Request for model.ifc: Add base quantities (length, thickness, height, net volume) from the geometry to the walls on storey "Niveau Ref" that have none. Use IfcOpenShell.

First a look at what the model holds.

```python
import ifcopenshell
import ifcopenshell.util.element
import ifcopenshell.util.unit

model = ifcopenshell.open("model.ifc")
print(model.schema)
for unit_type in ("LENGTHUNIT", "AREAUNIT", "VOLUMEUNIT"):
    print(unit_type, ifcopenshell.util.unit.calculate_unit_scale(model, unit_type))
storey = next(s for s in model.by_type("IfcBuildingStorey") if s.Name == "Niveau Ref")
walls = [e for e in ifcopenshell.util.element.get_decomposition(storey) if e.is_a("IfcWall")]
for e in sorted(walls, key=lambda e: e.id()):
    print(e.id(), e.is_a(), e.Name, list(ifcopenshell.util.element.get_psets(e, qtos_only=True)), sep=" | ")
```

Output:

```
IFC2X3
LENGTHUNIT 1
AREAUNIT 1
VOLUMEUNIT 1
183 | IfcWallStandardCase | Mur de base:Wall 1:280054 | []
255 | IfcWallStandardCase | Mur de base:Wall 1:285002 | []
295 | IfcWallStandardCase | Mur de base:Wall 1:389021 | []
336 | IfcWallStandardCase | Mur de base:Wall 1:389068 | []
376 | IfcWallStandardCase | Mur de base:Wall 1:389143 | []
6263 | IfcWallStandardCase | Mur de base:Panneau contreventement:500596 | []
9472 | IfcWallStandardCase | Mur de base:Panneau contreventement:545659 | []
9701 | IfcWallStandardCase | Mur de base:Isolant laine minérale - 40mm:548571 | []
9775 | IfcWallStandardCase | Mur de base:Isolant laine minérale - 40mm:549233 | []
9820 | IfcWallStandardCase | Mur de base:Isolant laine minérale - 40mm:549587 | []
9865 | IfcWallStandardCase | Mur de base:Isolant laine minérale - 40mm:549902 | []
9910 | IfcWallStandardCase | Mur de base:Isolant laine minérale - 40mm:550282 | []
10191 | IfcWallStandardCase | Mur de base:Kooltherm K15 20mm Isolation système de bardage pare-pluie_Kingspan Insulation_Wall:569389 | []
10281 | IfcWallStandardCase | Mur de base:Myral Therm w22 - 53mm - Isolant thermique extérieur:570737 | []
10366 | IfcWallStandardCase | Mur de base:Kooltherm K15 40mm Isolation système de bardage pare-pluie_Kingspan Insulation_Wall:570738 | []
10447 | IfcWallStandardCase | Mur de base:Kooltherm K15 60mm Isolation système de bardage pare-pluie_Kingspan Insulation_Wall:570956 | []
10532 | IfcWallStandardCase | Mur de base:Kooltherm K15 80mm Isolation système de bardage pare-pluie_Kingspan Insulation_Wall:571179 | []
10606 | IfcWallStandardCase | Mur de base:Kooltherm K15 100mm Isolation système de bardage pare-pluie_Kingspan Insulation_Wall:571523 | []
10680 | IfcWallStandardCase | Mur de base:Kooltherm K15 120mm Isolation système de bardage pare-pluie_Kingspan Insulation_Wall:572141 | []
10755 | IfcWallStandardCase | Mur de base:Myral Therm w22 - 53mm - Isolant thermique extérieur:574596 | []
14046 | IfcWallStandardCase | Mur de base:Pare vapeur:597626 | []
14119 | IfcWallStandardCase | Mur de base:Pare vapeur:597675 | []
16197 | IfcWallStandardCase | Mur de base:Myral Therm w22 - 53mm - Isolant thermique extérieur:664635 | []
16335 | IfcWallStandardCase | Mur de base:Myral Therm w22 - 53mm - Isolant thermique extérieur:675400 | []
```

```python
import ifcopenshell
import ifcopenshell.api.pset
import ifcopenshell.geom
import ifcopenshell.util.element
import ifcopenshell.util.shape
import ifcopenshell.util.unit

model = ifcopenshell.open("model.ifc")
unit_scale = ifcopenshell.util.unit.calculate_unit_scale(model)
volume_scale = ifcopenshell.util.unit.calculate_unit_scale(model, "VOLUMEUNIT")
settings = ifcopenshell.geom.settings()

storey = next(s for s in model.by_type("IfcBuildingStorey") if s.Name == "Niveau Ref")
walls = [e for e in ifcopenshell.util.element.get_decomposition(storey) if e.is_a("IfcWall")]

for e in sorted(walls, key=lambda e: e.id()):
    if ifcopenshell.util.element.get_psets(e, qtos_only=True, should_inherit=False):
        continue
    # Geometry comes back in metres, in the element's own axes.
    shape = ifcopenshell.geom.create_shape(settings, e)
    values = {
        "Length": ifcopenshell.util.shape.get_x(shape.geometry) / unit_scale,
        "Width": ifcopenshell.util.shape.get_y(shape.geometry) / unit_scale,
        "Height": ifcopenshell.util.shape.get_z(shape.geometry) / unit_scale,
        "NetVolume": ifcopenshell.util.shape.get_volume(shape.geometry) / volume_scale,
    }
    qto = ifcopenshell.api.pset.add_qto(model, product=e, name="BaseQuantities")
    ifcopenshell.api.pset.edit_qto(model, qto=qto, properties=values)
    print(e.id(), {k: round(v, 3) for k, v in values.items()})

model.write("model-out.ifc")
```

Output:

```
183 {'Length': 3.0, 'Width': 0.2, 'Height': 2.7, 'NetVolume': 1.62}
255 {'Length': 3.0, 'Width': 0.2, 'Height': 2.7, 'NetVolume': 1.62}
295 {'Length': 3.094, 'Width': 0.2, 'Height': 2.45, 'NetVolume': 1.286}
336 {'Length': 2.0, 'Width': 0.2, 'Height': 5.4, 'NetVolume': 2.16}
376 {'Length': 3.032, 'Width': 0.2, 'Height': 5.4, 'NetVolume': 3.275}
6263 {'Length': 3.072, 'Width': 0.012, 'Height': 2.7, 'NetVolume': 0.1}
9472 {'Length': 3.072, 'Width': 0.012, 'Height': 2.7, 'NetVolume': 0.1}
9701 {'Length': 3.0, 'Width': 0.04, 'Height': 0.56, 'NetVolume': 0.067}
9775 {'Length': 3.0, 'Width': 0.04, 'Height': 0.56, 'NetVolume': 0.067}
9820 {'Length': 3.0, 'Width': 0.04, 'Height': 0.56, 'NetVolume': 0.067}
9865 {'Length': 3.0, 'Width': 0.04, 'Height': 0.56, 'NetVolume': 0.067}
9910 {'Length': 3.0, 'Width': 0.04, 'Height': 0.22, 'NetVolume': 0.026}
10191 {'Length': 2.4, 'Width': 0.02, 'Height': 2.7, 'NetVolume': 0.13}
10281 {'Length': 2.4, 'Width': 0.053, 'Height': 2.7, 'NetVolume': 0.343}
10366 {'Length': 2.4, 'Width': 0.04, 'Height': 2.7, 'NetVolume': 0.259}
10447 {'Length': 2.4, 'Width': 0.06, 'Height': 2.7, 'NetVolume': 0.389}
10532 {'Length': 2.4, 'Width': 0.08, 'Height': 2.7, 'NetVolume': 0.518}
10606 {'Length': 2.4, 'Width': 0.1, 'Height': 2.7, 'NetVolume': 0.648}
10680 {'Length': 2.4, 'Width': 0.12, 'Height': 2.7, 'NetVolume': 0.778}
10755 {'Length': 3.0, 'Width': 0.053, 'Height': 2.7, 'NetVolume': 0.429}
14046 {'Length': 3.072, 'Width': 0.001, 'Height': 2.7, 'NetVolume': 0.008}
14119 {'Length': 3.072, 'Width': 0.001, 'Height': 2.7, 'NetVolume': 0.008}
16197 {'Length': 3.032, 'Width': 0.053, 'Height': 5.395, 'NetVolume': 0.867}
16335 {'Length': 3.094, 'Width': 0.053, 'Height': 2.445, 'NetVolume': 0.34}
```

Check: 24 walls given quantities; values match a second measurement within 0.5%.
